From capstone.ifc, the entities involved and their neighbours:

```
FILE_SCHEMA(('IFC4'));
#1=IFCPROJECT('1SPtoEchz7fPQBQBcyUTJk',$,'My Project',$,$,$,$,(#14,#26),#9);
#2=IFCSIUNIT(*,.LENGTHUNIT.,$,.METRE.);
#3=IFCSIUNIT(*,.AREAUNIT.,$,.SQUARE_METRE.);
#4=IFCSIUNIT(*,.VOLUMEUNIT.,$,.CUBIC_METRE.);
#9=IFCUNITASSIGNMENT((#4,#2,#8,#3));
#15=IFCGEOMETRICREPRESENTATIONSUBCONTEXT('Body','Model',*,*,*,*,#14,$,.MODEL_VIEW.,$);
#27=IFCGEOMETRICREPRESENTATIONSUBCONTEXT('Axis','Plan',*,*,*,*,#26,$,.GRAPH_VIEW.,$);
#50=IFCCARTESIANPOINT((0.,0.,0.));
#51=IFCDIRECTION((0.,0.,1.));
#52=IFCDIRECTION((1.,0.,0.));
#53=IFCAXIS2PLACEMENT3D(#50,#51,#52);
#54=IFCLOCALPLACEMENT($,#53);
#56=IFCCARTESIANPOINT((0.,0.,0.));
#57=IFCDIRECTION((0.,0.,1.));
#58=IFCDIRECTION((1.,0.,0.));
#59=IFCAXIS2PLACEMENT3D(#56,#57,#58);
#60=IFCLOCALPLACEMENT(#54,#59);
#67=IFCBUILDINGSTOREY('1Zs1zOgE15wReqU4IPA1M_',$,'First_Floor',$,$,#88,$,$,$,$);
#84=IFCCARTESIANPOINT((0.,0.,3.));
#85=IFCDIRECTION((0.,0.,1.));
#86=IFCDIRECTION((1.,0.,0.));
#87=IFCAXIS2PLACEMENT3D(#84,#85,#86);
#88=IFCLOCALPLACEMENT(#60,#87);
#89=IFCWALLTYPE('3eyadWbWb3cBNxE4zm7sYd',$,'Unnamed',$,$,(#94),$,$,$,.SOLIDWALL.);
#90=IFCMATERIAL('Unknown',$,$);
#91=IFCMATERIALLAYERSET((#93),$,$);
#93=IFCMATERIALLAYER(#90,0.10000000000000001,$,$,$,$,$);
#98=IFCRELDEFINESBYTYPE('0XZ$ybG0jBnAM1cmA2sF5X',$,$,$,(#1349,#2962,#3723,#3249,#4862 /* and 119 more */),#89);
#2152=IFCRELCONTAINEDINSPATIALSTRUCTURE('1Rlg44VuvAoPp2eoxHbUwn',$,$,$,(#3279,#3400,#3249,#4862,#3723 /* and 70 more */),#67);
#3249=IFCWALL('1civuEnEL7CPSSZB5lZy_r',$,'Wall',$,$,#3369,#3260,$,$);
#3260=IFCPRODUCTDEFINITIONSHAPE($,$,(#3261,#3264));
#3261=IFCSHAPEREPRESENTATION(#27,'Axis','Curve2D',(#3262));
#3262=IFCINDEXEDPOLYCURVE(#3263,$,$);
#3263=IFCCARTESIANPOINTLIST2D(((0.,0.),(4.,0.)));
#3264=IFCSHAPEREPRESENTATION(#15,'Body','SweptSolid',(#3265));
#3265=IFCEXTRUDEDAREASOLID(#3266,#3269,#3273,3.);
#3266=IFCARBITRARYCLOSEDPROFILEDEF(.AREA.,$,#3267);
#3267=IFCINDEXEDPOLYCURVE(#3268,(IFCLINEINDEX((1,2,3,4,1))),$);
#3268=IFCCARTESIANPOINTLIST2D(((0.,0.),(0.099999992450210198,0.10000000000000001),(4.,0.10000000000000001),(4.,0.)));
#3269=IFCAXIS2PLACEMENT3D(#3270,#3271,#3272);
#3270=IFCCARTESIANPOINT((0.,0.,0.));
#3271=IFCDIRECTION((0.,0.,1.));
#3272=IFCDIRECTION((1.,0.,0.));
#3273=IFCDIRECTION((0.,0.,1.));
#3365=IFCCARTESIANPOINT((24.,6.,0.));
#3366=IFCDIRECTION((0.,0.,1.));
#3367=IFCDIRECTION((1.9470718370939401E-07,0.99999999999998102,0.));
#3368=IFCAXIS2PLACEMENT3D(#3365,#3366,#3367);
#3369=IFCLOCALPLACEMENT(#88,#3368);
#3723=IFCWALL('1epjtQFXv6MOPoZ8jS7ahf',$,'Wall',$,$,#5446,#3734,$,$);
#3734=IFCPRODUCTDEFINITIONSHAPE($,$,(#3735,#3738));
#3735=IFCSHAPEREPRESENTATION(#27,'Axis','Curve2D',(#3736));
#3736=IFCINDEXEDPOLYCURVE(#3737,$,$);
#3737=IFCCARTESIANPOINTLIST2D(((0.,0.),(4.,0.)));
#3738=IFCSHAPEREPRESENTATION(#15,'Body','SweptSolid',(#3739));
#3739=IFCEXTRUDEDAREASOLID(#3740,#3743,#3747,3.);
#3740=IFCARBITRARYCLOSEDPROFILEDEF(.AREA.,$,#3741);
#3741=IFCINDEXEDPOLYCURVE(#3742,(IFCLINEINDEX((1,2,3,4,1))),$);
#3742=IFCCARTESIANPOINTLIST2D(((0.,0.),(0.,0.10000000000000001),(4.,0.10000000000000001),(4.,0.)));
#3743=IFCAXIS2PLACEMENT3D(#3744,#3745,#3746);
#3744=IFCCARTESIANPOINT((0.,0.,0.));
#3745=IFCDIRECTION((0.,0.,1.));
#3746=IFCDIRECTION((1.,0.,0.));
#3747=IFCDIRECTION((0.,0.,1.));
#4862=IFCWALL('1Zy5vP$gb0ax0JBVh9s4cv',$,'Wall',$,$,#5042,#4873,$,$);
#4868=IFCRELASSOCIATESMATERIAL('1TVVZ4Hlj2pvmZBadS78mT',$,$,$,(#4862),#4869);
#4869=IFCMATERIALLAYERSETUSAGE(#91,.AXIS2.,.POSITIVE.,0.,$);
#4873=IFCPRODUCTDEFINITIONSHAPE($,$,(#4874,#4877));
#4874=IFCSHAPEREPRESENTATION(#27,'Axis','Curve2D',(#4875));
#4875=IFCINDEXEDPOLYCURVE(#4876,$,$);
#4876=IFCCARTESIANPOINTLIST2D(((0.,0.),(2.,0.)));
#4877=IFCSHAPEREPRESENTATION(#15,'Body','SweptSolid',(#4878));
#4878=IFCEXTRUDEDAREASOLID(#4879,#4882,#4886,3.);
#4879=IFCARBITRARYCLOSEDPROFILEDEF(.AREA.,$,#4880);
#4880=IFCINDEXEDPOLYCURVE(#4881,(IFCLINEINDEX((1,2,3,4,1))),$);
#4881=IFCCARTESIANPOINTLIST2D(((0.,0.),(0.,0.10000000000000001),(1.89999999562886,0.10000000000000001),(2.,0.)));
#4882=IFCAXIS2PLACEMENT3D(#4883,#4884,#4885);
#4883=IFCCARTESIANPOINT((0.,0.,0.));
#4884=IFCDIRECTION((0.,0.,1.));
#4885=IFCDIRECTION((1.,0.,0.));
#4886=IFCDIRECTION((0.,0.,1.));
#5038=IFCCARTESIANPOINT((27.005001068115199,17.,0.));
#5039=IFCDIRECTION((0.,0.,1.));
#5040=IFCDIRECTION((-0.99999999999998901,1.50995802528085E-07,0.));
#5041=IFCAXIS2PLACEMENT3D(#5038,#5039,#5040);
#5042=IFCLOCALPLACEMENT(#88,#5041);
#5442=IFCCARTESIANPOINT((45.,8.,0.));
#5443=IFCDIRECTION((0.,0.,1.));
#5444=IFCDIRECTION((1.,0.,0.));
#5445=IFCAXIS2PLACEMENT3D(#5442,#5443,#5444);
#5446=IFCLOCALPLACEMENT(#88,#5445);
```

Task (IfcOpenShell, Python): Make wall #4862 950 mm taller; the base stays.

```python
import ifcopenshell
import ifcopenshell.geom
import ifcopenshell.util.representation
import ifcopenshell.util.shape
import ifcopenshell.util.unit

model = ifcopenshell.open("capstone.ifc")
unit_scale = ifcopenshell.util.unit.calculate_unit_scale(model)
settings = ifcopenshell.geom.settings()


def volume(element):
    """Net volume in cubic metres, openings subtracted."""
    shape = ifcopenshell.geom.create_shape(settings, element)
    return ifcopenshell.util.shape.get_volume(shape.geometry)


wall = model.by_guid("1Zy5vP$gb0ax0JBVh9s4cv")
before = volume(wall)

body = ifcopenshell.util.representation.get_representation(wall, "Model", "Body")
solid = body.Items[0]
old_height = solid.Depth
solid.Depth += 0.95 / unit_scale
after = volume(wall)

print(f"height {old_height:g} -> {solid.Depth:g}, volume {before:.3f} -> {after:.3f} m3")

model.write("capstone_rev.ifc")
```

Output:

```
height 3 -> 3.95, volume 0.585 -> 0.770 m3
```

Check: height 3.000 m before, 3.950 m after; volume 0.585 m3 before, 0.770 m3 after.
